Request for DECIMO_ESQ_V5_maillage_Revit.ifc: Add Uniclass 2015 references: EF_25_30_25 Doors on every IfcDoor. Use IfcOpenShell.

First a look at what the model holds.

```python
import ifcopenshell

model = ifcopenshell.open("DECIMO_ESQ_V5_maillage_Revit.ifc")
print(model.schema)
print("classifications:", [c.Name for c in model.by_type("IfcClassification")])
for ifc_class in ("IfcDoor", "IfcRoof", "IfcStair", "IfcWall", "IfcWindow"):
    print(ifc_class, len(model.by_type(ifc_class)))
```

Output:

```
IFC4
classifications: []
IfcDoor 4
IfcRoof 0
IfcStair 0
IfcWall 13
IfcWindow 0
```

```python
import ifcopenshell
import ifcopenshell.api.classification

model = ifcopenshell.open("DECIMO_ESQ_V5_maillage_Revit.ifc")

system = ifcopenshell.api.classification.add_classification(model, classification="Uniclass 2015")

codes = {
    "IfcDoor": ("EF_25_30_25", "Doors"),
}
for ifc_class, (code, name) in codes.items():
    products = model.by_type(ifc_class)
    ifcopenshell.api.classification.add_reference(
        model, products=products, classification=system, identification=code, name=name
    )
    print(code, len(products))

model.write("DECIMO_ESQ_V5_maillage_Revit_updated.ifc")
```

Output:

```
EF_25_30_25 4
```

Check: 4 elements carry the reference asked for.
